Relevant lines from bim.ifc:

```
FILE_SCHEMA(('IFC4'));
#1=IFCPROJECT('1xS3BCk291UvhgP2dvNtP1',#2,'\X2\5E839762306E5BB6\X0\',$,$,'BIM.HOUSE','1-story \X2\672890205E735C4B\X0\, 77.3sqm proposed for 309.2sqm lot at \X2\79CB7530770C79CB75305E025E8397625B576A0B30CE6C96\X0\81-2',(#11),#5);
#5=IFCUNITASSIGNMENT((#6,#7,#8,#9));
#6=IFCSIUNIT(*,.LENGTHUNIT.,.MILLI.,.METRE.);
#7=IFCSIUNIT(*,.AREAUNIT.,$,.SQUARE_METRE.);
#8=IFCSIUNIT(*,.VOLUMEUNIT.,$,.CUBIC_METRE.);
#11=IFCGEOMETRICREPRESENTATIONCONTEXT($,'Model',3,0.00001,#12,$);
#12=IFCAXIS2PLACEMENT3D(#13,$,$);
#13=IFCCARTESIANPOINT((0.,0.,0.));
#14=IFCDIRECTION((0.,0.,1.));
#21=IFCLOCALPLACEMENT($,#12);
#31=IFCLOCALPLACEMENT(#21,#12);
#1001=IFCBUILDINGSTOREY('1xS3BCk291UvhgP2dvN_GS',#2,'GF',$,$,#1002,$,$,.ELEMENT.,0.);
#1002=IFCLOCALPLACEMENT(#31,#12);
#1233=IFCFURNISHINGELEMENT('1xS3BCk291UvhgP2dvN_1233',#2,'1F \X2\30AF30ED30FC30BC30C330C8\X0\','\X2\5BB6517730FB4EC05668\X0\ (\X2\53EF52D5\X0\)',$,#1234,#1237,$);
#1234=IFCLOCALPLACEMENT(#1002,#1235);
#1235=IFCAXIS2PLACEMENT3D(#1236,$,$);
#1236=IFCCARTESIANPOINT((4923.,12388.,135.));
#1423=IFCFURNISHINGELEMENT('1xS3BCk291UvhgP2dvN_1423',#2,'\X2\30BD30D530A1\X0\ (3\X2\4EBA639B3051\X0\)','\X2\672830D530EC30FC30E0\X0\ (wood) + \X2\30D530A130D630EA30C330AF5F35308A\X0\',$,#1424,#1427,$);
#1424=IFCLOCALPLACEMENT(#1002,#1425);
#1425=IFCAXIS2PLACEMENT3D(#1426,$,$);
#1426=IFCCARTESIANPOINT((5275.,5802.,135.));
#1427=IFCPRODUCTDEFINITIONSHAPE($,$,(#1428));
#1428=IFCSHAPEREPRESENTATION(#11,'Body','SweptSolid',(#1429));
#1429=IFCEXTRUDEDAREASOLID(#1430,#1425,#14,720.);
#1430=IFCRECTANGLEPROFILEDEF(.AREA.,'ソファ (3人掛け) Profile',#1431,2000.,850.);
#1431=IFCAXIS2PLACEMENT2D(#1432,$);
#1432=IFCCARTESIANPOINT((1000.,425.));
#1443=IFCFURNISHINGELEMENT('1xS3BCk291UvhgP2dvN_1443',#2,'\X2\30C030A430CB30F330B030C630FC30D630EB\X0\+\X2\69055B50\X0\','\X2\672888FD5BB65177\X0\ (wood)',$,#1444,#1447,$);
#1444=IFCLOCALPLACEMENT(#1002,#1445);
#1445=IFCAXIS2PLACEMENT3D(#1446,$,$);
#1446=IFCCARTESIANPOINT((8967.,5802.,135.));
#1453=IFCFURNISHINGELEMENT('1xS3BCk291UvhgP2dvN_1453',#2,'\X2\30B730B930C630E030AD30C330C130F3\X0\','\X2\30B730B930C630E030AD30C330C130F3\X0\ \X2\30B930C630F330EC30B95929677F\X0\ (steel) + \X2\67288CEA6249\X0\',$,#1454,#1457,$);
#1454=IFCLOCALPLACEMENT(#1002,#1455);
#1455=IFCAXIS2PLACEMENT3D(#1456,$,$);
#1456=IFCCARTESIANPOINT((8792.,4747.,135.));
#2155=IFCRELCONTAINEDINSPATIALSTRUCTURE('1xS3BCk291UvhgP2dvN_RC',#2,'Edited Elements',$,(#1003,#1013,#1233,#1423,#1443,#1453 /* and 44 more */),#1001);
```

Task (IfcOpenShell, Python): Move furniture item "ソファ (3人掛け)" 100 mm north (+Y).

```python
import ifcopenshell
import ifcopenshell.api.geometry
import ifcopenshell.util.placement
import ifcopenshell.util.unit

model = ifcopenshell.open("bim.ifc")
unit_scale = ifcopenshell.util.unit.calculate_unit_scale(model)

item = model.by_id(1423)
matrix = ifcopenshell.util.placement.get_local_placement(item.ObjectPlacement)
matrix[1, 3] += 0.1 / unit_scale
ifcopenshell.api.geometry.edit_object_placement(model, product=item, matrix=matrix, is_si=False)

print(ifcopenshell.util.placement.get_local_placement(item.ObjectPlacement).round(3) + 0.0)

model.write("bim_rev.ifc")
```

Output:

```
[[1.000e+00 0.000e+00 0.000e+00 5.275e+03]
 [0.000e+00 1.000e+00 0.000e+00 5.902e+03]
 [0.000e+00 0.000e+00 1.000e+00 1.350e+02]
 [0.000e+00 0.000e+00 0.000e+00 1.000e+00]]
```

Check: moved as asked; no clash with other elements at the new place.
